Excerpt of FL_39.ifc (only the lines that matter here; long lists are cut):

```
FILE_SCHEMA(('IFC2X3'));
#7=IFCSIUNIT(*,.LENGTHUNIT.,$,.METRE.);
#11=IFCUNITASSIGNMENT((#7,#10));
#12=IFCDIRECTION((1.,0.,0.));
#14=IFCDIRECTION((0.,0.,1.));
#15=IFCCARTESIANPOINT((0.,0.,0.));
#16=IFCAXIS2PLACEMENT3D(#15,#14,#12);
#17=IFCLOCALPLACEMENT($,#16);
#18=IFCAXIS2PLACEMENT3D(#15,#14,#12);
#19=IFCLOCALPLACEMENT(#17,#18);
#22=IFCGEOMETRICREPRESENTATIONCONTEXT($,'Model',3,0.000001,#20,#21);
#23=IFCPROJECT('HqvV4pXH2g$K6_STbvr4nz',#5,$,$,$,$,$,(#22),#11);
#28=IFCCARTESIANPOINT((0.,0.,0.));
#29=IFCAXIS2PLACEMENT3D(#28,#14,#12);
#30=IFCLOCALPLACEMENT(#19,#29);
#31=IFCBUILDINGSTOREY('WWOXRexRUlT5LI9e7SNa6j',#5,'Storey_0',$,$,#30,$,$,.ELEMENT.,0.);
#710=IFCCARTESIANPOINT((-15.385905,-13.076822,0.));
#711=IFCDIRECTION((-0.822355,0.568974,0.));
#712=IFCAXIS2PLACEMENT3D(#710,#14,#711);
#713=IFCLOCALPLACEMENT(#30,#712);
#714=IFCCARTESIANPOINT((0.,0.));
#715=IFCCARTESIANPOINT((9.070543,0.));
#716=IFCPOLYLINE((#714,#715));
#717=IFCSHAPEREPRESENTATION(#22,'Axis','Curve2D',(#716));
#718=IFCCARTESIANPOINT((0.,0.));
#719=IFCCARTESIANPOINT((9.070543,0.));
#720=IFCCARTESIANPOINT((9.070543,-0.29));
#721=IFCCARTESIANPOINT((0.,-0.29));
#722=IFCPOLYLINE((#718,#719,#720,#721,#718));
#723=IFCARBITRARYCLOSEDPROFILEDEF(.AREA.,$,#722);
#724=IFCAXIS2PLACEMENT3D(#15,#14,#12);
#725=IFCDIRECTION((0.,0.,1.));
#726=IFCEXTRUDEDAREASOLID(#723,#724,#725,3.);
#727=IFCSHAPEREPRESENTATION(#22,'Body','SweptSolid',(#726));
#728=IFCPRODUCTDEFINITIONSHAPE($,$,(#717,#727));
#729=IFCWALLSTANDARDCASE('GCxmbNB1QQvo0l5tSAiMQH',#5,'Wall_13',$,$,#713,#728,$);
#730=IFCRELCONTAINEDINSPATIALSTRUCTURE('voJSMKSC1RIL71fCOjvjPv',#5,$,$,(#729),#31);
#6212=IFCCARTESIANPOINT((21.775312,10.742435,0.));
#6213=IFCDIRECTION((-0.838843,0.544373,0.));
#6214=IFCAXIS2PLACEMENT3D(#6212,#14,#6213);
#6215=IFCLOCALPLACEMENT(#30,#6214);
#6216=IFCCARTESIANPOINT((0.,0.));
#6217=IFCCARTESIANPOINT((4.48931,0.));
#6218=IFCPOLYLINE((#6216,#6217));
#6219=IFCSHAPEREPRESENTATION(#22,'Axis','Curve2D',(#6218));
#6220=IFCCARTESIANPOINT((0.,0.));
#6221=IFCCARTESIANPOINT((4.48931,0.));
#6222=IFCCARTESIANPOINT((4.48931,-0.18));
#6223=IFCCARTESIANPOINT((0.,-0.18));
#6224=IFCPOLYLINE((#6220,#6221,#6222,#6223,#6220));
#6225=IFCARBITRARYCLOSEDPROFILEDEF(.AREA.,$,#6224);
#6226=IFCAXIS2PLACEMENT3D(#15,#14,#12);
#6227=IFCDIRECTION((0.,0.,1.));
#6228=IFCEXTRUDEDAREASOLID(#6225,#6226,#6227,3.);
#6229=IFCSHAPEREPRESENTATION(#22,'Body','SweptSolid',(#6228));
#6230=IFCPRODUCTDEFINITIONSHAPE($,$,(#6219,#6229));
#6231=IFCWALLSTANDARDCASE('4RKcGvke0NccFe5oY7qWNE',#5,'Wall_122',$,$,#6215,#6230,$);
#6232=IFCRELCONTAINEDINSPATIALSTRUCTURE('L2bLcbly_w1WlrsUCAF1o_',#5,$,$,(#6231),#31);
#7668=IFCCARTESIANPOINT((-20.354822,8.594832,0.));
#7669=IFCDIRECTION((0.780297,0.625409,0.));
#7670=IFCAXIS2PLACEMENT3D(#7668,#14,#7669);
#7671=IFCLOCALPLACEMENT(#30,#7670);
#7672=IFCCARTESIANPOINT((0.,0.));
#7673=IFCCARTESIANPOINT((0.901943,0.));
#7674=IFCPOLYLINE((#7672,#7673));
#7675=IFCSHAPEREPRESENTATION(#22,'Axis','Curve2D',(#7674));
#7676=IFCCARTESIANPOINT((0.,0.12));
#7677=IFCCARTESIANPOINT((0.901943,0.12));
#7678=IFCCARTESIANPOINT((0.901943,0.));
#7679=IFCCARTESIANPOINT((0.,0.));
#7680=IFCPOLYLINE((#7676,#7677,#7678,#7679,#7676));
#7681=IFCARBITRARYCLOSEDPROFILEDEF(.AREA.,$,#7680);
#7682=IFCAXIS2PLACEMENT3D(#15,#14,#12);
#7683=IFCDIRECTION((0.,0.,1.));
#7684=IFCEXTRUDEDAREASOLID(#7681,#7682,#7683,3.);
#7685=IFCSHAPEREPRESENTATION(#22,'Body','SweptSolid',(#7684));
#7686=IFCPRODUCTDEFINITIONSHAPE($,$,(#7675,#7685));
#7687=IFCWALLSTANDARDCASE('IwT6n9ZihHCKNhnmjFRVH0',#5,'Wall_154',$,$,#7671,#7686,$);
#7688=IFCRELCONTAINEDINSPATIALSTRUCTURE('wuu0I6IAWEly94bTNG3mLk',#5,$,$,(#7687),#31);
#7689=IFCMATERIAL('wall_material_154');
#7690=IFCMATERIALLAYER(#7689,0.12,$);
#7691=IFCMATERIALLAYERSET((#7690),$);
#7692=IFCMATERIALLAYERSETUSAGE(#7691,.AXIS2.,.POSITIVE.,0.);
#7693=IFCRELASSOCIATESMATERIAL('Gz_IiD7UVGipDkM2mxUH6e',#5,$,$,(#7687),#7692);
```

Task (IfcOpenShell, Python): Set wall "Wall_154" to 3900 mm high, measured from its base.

```python
import ifcopenshell
import ifcopenshell.geom
import ifcopenshell.util.shape

model = ifcopenshell.open("FL_39.ifc")
settings = ifcopenshell.geom.settings()


def volume(element):
    """Net volume in cubic metres, openings subtracted."""
    shape = ifcopenshell.geom.create_shape(settings, element)
    return ifcopenshell.util.shape.get_volume(shape.geometry)


wall = model.by_guid("IwT6n9ZihHCKNhnmjFRVH0")
before = volume(wall)

body = next(r for r in wall.Representation.Representations if r.RepresentationIdentifier == "Body")
solid = body.Items[0]
old_height = solid.Depth
solid.Depth = 3.9
after = volume(wall)

print(f"height {old_height:g} -> {solid.Depth:g}, volume {before:.3f} -> {after:.3f} m3")

model.write("FL_39_updated.ifc")
```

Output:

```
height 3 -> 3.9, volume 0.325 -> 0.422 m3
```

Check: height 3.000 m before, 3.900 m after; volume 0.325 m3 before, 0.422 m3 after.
